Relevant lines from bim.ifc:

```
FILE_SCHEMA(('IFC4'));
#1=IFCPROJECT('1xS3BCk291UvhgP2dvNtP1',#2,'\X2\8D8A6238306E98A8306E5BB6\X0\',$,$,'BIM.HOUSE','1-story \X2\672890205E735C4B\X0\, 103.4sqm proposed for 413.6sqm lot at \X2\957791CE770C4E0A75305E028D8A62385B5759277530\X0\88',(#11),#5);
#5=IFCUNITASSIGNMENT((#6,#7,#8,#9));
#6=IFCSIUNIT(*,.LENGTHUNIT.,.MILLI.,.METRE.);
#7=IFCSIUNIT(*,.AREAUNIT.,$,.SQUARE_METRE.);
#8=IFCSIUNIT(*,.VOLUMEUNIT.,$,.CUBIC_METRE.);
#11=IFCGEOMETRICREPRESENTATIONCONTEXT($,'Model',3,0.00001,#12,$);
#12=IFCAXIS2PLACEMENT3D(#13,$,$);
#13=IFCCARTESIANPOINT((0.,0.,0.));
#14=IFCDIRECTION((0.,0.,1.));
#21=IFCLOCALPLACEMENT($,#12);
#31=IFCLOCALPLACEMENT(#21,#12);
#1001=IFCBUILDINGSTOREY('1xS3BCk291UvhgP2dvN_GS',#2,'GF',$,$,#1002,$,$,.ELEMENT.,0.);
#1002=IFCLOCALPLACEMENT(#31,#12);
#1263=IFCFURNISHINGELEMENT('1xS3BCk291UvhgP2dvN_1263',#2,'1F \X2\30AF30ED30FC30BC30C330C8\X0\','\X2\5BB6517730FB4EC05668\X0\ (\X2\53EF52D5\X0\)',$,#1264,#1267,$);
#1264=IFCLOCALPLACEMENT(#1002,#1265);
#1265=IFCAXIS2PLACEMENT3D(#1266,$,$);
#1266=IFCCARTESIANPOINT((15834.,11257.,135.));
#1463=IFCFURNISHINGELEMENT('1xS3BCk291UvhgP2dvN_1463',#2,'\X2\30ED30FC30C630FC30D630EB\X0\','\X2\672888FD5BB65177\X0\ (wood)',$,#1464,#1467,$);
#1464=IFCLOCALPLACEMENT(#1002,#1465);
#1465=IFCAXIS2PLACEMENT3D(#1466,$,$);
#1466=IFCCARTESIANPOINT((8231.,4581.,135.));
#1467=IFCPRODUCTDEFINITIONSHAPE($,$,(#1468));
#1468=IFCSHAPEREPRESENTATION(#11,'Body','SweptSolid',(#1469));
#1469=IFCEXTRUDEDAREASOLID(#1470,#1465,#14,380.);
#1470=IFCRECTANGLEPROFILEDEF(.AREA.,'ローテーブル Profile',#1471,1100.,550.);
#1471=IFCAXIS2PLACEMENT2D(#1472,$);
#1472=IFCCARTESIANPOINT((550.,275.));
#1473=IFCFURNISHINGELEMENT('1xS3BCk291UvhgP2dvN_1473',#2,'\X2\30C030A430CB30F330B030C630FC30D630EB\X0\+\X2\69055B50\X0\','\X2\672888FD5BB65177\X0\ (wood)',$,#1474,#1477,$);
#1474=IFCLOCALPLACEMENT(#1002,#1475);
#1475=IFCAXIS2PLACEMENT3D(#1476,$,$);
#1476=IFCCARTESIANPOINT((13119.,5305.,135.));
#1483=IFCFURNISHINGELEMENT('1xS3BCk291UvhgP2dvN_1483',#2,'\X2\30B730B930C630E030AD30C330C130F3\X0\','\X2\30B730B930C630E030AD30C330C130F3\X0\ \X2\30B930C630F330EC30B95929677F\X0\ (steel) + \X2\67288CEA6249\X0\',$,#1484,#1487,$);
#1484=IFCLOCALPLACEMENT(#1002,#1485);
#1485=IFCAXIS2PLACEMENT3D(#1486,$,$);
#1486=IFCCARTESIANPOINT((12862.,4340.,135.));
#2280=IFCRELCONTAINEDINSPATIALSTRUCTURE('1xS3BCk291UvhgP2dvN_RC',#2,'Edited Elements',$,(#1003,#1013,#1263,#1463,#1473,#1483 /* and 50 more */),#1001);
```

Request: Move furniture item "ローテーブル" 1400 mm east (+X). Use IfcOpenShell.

```python
import ifcopenshell
import ifcopenshell.api.geometry
import ifcopenshell.util.placement

model = ifcopenshell.open("bim.ifc")

item = model.by_id(1463)
matrix = ifcopenshell.util.placement.get_local_placement(item.ObjectPlacement)
matrix[0, 3] += 1400.0
ifcopenshell.api.geometry.edit_object_placement(model, product=item, matrix=matrix, is_si=False)

print(ifcopenshell.util.placement.get_local_placement(item.ObjectPlacement).round(3) + 0.0)

model.write("bim_edited.ifc")
```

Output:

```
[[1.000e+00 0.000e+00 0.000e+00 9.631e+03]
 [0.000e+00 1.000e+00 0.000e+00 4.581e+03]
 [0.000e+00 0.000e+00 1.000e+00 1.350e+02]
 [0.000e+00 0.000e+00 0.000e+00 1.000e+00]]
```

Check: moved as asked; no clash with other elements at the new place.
